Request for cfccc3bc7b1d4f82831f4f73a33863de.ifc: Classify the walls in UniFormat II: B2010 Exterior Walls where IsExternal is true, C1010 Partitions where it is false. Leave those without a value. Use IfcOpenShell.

First a look at what the model holds.

```python
import ifcopenshell
import ifcopenshell.util.element

model = ifcopenshell.open("cfccc3bc7b1d4f82831f4f73a33863de.ifc")
print(model.schema)
print("classifications:", [c.Name for c in model.by_type("IfcClassification")])
values = [ifcopenshell.util.element.get_pset(e, "Pset_WallCommon", "IsExternal") for e in model.by_type("IfcWall")]
for value in (True, False, None):
    print("IsExternal", value, values.count(value))
```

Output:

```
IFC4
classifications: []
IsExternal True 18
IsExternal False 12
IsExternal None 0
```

```python
import ifcopenshell
import ifcopenshell.api.classification
import ifcopenshell.util.element

model = ifcopenshell.open("cfccc3bc7b1d4f82831f4f73a33863de.ifc")

system = ifcopenshell.api.classification.add_classification(model, classification="UniFormat II")

walls = model.by_type("IfcWall")
external = {e: ifcopenshell.util.element.get_pset(e, "Pset_WallCommon", "IsExternal") for e in walls}
for flag, code, name in ((True, "B2010", "Exterior Walls"), (False, "C1010", "Partitions")):
    products = [e for e in walls if external[e] is flag]
    ifcopenshell.api.classification.add_reference(
        model, products=products, classification=system, identification=code, name=name
    )
    print(code, len(products))

model.write("cfccc3bc7b1d4f82831f4f73a33863de_rev.ifc")
```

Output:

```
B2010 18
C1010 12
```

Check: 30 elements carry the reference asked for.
